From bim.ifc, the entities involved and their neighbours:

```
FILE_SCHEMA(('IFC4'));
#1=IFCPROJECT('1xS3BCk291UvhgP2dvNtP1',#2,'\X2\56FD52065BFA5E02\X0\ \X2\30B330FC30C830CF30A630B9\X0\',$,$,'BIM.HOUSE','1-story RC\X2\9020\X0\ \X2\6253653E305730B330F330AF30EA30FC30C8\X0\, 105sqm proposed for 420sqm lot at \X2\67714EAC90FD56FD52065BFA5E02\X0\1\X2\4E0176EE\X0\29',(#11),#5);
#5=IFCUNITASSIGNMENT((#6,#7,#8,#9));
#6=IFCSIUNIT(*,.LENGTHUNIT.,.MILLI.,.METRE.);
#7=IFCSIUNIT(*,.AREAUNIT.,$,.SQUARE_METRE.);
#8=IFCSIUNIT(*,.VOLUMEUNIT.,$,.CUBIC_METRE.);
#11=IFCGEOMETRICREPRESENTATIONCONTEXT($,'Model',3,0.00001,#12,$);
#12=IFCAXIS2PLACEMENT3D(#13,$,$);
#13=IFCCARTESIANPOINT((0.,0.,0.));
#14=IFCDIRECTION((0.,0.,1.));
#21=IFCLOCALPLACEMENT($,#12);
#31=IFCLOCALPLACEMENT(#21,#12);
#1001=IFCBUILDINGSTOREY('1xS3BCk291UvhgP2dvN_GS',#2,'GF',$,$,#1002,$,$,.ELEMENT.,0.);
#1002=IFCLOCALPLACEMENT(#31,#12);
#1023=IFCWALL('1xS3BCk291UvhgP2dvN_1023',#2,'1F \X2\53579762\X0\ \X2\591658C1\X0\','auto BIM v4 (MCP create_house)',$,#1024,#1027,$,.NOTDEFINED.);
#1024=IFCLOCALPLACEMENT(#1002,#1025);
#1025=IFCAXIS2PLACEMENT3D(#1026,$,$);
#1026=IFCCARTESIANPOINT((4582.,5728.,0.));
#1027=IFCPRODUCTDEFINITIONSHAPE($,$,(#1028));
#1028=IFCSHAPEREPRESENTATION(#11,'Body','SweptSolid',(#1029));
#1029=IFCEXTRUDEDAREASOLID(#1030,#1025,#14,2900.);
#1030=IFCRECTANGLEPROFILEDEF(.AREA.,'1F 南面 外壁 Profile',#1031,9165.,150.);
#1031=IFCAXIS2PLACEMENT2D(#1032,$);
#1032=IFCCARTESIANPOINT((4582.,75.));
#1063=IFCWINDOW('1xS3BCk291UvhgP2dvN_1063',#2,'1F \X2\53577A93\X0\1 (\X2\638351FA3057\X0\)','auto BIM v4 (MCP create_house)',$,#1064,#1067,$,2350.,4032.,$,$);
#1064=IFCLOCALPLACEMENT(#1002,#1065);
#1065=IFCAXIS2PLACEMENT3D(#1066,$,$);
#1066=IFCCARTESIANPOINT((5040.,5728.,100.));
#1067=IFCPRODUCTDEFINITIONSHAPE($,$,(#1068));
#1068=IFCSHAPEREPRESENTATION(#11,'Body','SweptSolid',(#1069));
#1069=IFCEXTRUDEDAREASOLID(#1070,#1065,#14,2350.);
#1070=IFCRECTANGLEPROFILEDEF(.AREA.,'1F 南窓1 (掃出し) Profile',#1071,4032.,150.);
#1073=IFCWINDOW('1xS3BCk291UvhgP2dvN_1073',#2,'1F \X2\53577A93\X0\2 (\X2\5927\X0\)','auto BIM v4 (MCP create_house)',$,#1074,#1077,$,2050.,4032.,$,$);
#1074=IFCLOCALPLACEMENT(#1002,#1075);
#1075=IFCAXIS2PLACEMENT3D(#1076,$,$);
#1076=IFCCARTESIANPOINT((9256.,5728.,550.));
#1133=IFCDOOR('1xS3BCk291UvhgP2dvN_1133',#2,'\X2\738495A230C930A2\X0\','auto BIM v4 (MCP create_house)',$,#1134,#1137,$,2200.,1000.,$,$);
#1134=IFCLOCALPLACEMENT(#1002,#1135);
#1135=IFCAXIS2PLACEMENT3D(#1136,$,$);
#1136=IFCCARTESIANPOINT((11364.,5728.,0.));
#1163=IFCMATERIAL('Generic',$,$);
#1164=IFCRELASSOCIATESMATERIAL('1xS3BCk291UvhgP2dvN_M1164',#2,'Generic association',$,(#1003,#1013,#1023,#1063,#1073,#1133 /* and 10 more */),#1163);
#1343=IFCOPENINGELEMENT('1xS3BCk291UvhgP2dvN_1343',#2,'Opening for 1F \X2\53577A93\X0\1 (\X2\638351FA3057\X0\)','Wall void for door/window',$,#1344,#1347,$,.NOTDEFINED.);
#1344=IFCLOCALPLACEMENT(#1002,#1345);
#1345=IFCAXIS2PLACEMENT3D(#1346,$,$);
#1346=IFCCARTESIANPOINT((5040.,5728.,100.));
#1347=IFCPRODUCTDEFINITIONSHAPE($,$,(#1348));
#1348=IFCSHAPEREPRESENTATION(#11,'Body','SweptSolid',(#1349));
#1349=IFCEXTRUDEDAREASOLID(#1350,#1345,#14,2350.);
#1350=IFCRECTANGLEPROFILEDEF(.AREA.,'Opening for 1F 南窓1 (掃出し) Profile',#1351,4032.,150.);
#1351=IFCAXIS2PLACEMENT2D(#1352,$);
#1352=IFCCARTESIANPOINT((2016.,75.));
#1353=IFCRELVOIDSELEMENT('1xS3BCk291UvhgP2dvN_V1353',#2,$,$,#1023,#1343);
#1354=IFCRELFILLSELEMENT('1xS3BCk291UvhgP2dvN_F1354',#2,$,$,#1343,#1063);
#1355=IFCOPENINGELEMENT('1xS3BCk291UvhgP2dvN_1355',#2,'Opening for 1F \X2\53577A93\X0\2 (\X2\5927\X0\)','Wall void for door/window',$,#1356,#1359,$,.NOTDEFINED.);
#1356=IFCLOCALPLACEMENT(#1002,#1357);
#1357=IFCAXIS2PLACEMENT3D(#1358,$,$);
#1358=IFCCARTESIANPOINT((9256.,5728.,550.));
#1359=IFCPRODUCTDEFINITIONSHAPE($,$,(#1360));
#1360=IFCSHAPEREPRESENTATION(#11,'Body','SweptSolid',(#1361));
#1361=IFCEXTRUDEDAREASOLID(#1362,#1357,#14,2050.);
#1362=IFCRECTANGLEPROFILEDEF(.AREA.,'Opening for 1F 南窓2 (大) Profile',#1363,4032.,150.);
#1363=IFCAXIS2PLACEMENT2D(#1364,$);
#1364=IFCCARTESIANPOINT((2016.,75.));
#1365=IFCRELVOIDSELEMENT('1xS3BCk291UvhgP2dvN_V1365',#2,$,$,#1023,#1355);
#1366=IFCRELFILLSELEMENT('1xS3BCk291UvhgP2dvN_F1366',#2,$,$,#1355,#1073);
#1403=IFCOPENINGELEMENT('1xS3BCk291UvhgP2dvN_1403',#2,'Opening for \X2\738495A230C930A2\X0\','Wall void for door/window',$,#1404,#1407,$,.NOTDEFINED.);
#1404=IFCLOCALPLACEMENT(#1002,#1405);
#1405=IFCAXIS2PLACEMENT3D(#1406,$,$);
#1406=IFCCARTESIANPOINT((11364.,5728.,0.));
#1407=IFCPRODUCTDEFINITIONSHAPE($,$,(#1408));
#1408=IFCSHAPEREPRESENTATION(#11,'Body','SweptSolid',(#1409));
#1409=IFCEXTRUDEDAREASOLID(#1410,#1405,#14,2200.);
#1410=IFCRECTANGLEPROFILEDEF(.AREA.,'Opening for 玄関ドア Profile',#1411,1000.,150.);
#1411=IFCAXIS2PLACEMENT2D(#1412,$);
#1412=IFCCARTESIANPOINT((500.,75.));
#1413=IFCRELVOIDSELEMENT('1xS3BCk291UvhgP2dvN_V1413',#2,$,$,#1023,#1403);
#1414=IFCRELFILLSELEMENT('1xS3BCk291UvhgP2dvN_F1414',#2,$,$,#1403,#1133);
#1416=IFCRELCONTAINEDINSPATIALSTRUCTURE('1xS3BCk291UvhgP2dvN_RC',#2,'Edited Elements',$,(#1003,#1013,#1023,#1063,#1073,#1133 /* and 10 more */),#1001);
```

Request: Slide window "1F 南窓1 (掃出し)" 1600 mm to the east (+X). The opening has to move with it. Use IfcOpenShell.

```python
import ifcopenshell
import ifcopenshell.api.geometry
import ifcopenshell.util.placement

model = ifcopenshell.open("bim.ifc")

window = model.by_guid("1xS3BCk291UvhgP2dvN_1063")
opening = window.FillsVoids[0].RelatingOpeningElement
wall = opening.VoidsElements[0].RelatingBuildingElement

wall_matrix = ifcopenshell.util.placement.get_local_placement(wall.ObjectPlacement)
shift = wall_matrix[:3, 0] * 1600.0
before = ifcopenshell.util.placement.get_local_placement(window.ObjectPlacement)[:3, 3].copy()

# The window is not placed relative to its opening, so move both.
for product in (opening, window):
    matrix = ifcopenshell.util.placement.get_local_placement(product.ObjectPlacement)
    matrix[:3, 3] += shift
    ifcopenshell.api.geometry.edit_object_placement(model, product=product, matrix=matrix, is_si=False)

after = ifcopenshell.util.placement.get_local_placement(window.ObjectPlacement)[:3, 3]
print("window moved by", (after - before).round(3) + 0.0)

model.write("bim_rev.ifc")
```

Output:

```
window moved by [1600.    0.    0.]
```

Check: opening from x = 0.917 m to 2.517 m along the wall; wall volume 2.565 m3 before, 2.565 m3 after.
